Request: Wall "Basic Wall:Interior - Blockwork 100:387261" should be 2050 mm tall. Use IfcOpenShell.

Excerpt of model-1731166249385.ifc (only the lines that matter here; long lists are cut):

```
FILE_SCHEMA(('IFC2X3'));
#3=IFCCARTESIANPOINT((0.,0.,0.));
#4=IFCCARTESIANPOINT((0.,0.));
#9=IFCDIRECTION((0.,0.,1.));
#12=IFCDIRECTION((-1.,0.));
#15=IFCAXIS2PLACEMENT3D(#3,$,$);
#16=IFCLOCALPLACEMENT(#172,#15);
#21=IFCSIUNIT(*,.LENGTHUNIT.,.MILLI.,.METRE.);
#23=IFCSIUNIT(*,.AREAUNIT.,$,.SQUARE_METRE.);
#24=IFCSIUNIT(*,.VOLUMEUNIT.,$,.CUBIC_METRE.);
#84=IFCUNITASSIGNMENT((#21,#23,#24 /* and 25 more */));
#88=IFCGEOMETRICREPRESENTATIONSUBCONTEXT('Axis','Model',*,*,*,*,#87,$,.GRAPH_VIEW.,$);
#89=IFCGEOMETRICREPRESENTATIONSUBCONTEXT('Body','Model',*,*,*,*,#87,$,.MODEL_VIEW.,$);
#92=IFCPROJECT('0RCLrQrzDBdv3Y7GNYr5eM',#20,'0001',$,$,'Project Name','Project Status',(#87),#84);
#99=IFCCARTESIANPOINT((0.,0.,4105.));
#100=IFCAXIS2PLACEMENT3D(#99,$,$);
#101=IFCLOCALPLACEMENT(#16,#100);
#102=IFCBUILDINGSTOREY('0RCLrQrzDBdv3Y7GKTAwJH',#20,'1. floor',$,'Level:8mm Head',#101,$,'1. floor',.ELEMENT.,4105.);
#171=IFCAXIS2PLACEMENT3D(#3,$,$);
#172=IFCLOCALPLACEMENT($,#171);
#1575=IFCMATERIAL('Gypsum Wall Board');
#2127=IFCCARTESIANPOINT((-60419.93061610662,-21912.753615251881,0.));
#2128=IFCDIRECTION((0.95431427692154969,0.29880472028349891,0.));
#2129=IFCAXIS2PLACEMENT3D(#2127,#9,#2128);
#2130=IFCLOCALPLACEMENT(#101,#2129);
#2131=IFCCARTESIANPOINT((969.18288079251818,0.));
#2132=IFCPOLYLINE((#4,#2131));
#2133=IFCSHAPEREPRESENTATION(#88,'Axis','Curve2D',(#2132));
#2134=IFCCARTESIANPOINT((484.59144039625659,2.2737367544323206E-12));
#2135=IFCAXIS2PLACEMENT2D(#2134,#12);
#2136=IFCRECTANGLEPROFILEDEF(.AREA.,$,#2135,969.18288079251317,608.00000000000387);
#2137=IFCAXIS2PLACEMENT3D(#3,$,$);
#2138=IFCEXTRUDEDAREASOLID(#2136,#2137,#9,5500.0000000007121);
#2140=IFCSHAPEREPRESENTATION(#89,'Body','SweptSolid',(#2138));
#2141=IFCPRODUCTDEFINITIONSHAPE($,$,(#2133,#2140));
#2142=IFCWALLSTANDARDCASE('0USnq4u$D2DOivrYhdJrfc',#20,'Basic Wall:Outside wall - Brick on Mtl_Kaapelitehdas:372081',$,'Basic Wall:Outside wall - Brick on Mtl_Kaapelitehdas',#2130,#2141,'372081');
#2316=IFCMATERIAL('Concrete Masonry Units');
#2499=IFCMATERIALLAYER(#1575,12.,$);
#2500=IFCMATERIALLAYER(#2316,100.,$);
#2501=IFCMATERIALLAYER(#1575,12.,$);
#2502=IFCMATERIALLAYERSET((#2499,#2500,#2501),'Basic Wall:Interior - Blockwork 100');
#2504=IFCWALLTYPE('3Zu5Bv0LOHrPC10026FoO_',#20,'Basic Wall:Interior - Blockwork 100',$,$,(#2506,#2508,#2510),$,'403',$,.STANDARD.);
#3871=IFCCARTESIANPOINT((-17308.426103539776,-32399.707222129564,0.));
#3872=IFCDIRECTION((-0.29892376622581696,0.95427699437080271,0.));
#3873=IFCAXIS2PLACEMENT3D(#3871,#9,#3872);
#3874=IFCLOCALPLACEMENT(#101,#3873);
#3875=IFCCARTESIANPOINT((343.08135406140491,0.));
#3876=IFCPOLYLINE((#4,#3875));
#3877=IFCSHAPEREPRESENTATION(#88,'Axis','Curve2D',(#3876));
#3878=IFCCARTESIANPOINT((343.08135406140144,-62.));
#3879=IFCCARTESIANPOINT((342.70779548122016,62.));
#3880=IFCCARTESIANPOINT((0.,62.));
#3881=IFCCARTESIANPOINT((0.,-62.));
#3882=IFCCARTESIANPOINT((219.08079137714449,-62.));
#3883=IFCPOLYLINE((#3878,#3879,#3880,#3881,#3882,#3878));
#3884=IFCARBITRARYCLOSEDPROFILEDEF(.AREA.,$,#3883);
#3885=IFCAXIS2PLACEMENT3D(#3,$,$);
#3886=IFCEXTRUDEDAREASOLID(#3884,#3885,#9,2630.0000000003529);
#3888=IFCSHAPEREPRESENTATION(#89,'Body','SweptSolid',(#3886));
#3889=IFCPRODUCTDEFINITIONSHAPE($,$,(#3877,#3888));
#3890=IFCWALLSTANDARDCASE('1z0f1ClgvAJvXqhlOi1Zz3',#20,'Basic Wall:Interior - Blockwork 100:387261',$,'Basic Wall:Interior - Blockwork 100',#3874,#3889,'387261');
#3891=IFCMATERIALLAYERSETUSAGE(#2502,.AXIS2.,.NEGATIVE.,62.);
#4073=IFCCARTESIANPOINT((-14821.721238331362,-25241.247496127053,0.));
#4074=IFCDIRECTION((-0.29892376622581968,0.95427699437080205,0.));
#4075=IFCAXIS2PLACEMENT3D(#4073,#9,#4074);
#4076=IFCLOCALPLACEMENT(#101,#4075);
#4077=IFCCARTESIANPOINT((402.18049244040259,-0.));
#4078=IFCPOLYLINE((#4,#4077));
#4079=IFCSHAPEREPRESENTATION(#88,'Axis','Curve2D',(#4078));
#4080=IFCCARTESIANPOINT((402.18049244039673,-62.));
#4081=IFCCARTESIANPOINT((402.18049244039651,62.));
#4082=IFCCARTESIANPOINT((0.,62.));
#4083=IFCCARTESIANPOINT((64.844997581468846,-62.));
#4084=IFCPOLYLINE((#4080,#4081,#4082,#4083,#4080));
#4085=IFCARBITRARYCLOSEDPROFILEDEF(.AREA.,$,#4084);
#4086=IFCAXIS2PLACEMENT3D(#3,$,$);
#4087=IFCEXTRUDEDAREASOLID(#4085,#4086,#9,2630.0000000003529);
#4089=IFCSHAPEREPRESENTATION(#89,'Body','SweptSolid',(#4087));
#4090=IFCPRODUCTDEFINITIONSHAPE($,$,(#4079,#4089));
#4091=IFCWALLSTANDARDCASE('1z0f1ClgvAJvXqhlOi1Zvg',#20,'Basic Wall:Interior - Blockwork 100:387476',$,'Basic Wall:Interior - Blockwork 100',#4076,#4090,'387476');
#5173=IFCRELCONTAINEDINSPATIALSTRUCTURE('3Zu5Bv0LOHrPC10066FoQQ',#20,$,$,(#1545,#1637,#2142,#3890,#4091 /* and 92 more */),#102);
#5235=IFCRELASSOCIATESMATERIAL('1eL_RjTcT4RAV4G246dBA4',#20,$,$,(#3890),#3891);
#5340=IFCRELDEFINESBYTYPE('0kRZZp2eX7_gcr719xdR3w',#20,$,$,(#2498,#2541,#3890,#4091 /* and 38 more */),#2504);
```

```python
import ifcopenshell
import ifcopenshell.geom
import ifcopenshell.util.representation
import ifcopenshell.util.shape
import ifcopenshell.util.unit

model = ifcopenshell.open("model-1731166249385.ifc")
unit_scale = ifcopenshell.util.unit.calculate_unit_scale(model)
settings = ifcopenshell.geom.settings()


def volume(element):
    """Net volume in cubic metres, openings subtracted."""
    shape = ifcopenshell.geom.create_shape(settings, element)
    return ifcopenshell.util.shape.get_volume(shape.geometry)


wall = model.by_guid("1z0f1ClgvAJvXqhlOi1Zz3")
before = volume(wall)

body = ifcopenshell.util.representation.get_representation(wall, "Model", "Body")
solid = body.Items[0]
old_height = solid.Depth
solid.Depth = 2.05 / unit_scale
after = volume(wall)

print(f"height {old_height:g} -> {solid.Depth:g}, volume {before:.3f} -> {after:.3f} m3")

model.write("model-1731166249385_edited.ifc")
```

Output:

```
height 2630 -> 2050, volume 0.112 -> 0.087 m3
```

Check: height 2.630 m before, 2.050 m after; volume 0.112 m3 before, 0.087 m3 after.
